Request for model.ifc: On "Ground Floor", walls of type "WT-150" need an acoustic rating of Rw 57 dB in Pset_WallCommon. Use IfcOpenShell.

First a look at what the model holds.

```python
import ifcopenshell
import ifcopenshell.util.element

model = ifcopenshell.open("model.ifc")
print(model.schema)
storey = next(s for s in model.by_type("IfcBuildingStorey") if s.Name == "Ground Floor")
walls = [e for e in ifcopenshell.util.element.get_decomposition(storey) if e.is_a("IfcWall")]
seen = {}
for e in walls:
    element_type = ifcopenshell.util.element.get_type(e)
    key = (element_type.Name if element_type != e and element_type else None, ifcopenshell.util.element.get_pset(e, "Pset_WallCommon", "AcousticRating"))
    seen[key] = seen.get(key, 0) + 1
for (name, value), count in sorted(seen.items(), key=str):
    print(count, "x", name, "|", value)
```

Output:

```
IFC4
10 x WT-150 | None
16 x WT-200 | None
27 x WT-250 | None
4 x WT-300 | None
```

```python
import ifcopenshell
import ifcopenshell.api.pset
import ifcopenshell.util.element

model = ifcopenshell.open("model.ifc")

storey = next(s for s in model.by_type("IfcBuildingStorey") if s.Name == "Ground Floor")
walls = [e for e in ifcopenshell.util.element.get_decomposition(storey) if e.is_a("IfcWall")]

count = 0
for e in walls:
    element_type = ifcopenshell.util.element.get_type(e)
    if element_type in (None, e) or element_type.Name != "WT-150":
        continue
    # add_pset returns the element's existing set when there is one.
    pset = ifcopenshell.api.pset.add_pset(model, product=e, name="Pset_WallCommon")
    ifcopenshell.api.pset.edit_pset(model, pset=pset, properties={"AcousticRating": "Rw 57 dB"})
    count += 1

print(count, "walls updated")

model.write("model_v2.ifc")
```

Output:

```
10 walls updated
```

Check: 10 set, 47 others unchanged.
